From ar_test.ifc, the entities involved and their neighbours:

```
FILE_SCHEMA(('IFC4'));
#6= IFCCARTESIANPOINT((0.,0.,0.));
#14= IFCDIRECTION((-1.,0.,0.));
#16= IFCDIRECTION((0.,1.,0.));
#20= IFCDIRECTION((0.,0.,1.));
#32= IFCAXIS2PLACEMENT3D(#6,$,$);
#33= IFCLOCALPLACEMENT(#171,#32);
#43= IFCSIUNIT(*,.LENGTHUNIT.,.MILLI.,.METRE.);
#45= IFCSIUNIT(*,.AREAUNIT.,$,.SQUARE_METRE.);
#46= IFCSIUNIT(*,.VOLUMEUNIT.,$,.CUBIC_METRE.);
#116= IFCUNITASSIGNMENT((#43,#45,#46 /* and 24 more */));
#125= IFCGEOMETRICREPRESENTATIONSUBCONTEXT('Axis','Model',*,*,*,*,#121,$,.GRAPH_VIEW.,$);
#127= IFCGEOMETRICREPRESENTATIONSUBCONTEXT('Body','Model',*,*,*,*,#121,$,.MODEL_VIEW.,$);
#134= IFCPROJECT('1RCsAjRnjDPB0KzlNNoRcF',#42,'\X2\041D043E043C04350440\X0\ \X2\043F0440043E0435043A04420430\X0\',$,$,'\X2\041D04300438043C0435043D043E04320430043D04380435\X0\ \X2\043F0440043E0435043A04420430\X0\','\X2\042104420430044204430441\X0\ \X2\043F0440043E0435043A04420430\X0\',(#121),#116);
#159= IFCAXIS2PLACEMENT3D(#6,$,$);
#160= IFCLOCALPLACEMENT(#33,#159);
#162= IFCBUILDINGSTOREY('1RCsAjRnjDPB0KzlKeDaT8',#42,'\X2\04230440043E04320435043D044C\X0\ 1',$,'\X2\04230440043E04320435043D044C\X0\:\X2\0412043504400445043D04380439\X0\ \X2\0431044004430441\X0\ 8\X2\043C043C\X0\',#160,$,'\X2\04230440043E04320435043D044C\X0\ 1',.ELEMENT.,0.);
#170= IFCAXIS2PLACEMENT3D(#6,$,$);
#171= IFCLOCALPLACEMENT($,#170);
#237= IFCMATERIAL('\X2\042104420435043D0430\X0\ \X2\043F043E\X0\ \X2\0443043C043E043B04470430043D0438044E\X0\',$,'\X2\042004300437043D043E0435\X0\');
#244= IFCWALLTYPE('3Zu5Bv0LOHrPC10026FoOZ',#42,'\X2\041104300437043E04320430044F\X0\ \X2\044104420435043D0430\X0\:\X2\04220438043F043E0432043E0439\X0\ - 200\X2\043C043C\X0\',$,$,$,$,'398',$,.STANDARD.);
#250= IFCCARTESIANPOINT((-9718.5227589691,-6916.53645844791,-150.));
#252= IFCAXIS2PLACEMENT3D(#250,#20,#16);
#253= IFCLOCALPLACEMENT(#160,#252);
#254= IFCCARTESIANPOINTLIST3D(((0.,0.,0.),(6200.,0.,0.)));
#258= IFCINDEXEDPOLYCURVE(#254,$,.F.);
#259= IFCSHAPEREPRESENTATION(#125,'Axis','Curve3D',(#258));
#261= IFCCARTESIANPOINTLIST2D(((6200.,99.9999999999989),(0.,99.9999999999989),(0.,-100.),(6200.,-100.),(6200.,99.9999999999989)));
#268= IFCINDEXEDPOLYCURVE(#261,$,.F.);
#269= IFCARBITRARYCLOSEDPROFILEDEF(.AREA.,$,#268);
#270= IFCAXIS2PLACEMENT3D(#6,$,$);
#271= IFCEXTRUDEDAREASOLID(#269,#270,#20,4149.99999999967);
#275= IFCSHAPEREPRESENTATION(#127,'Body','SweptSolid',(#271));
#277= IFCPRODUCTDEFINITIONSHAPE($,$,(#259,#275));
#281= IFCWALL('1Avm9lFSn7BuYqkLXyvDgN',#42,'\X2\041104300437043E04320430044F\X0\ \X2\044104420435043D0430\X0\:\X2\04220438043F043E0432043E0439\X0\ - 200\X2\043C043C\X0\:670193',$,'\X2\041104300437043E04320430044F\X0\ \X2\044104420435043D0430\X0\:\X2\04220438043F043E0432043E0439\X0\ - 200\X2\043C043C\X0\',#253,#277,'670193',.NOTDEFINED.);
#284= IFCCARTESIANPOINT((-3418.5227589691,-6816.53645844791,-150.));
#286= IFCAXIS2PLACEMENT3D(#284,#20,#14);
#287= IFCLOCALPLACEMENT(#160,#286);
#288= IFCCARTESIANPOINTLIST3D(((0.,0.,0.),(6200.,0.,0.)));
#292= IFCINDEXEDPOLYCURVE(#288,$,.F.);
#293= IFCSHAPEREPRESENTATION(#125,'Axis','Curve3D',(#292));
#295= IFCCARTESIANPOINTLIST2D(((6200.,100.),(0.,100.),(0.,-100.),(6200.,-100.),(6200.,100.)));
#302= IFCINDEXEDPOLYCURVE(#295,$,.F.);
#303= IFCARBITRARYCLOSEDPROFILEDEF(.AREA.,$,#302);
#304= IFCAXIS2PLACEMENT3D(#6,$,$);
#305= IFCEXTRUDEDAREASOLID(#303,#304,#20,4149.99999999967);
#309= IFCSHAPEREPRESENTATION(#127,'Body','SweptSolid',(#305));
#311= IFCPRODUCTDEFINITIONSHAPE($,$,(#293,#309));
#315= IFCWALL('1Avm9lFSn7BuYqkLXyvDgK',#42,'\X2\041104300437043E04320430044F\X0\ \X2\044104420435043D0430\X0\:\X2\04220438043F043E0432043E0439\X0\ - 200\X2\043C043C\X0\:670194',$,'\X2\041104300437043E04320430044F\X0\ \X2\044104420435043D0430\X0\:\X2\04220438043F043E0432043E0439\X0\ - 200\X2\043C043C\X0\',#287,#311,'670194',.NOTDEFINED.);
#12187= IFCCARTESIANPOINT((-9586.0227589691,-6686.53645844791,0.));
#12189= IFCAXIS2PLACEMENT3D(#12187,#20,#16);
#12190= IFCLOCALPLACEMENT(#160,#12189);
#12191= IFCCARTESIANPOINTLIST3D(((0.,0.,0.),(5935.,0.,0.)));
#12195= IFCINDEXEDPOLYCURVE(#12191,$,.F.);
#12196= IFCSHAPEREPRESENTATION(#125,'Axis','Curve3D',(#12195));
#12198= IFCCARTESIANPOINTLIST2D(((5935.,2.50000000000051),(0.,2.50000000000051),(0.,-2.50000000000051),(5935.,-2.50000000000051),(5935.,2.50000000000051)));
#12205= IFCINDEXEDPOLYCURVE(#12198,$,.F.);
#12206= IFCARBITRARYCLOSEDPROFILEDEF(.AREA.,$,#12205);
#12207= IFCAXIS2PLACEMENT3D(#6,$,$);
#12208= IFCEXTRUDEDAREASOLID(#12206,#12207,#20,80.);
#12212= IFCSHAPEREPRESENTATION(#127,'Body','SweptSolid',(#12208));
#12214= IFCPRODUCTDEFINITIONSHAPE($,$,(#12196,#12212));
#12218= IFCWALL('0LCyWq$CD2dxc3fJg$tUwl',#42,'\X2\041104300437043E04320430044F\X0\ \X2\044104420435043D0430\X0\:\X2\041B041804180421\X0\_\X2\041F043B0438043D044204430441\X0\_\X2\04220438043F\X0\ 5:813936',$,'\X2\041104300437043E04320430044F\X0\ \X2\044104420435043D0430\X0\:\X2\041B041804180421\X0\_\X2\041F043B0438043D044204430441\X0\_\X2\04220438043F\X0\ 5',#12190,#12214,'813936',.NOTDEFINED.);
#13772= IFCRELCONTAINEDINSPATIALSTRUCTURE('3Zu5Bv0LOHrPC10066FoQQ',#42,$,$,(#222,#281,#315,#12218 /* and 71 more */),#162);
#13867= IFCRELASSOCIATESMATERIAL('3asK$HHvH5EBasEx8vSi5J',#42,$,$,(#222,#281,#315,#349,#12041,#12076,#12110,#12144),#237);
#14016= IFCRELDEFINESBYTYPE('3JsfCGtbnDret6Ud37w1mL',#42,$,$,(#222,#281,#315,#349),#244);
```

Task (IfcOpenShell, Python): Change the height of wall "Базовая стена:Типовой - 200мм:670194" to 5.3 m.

```python
import ifcopenshell
import ifcopenshell.geom
import ifcopenshell.util.representation
import ifcopenshell.util.shape
import ifcopenshell.util.unit

model = ifcopenshell.open("ar_test.ifc")
unit_scale = ifcopenshell.util.unit.calculate_unit_scale(model)
settings = ifcopenshell.geom.settings()


def volume(element):
    """Net volume in cubic metres, openings subtracted."""
    shape = ifcopenshell.geom.create_shape(settings, element)
    return ifcopenshell.util.shape.get_volume(shape.geometry)


wall = model.by_id(315)
before = volume(wall)

body = ifcopenshell.util.representation.get_representation(wall, "Model", "Body")
solid = body.Items[0]
old_height = solid.Depth
solid.Depth = 5.3 / unit_scale
after = volume(wall)

print(f"height {old_height:g} -> {solid.Depth:g}, volume {before:.3f} -> {after:.3f} m3")

model.write("ar_test_v2.ifc")
```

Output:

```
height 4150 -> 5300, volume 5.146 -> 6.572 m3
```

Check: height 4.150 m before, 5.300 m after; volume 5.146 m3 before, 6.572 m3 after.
